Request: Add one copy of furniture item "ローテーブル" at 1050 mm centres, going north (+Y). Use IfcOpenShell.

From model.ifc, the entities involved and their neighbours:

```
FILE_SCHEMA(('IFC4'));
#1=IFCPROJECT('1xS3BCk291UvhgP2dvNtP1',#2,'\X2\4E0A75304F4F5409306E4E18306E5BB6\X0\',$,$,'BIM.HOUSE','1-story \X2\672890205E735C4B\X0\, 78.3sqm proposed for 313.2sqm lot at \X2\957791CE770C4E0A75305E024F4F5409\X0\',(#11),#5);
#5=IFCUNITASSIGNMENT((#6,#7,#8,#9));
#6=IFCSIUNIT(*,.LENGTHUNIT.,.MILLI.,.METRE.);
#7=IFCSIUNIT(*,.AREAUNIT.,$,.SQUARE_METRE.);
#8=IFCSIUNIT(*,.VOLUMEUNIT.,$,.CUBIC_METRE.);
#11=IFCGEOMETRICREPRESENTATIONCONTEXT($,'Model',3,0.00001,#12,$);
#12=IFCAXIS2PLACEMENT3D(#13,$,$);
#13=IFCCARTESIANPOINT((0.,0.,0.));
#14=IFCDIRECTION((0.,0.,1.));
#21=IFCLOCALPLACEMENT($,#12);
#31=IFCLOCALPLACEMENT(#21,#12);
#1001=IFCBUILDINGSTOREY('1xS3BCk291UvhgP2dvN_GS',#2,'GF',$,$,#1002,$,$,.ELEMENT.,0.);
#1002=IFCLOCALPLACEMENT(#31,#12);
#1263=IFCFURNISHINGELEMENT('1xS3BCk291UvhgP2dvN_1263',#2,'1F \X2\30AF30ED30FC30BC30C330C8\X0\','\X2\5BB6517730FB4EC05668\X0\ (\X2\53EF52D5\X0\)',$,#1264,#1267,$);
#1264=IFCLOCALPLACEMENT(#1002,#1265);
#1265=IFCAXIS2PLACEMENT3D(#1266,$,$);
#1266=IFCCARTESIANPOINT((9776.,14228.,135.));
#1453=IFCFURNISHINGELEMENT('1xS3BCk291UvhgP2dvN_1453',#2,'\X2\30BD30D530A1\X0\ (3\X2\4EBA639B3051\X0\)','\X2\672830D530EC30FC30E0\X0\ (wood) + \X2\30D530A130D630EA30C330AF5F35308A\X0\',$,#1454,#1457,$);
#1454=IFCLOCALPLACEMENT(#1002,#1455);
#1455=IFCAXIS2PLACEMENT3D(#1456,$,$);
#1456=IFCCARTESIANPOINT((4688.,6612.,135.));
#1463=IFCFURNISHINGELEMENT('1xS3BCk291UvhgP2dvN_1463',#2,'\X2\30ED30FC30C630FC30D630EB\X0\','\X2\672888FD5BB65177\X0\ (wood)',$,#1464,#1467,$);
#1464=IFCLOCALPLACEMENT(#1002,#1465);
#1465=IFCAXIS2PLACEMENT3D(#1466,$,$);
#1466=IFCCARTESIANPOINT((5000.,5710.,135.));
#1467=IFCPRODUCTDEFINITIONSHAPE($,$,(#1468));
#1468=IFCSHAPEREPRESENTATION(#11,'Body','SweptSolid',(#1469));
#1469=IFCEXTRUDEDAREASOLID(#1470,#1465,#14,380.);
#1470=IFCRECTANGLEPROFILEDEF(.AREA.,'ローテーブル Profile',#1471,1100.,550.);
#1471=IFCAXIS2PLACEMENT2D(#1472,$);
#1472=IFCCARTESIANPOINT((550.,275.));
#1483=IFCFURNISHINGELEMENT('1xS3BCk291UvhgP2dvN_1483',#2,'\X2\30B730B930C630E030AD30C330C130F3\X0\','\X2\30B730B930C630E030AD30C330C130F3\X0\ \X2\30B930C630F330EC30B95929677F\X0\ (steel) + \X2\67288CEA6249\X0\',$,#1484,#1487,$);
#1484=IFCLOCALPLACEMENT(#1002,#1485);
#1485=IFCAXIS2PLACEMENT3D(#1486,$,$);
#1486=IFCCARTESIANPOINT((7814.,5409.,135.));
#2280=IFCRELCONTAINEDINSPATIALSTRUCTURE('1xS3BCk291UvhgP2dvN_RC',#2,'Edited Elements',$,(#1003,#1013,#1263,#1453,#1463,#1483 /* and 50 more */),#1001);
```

```python
import numpy as np
import ifcopenshell
import ifcopenshell.api.geometry
import ifcopenshell.api.root
import ifcopenshell.util.element
import ifcopenshell.util.placement
import ifcopenshell.util.unit

model = ifcopenshell.open("model.ifc")
unit_scale = ifcopenshell.util.unit.calculate_unit_scale(model)


def reuse_history(source, copy):
    """copy_class also copies each property set's owner history, people and application; keep the originals."""
    for rel in copy.IsDefinedBy:
        if rel.is_a("IfcRelDefinesByProperties") and (history := rel.RelatingPropertyDefinition.OwnerHistory):
            rel.RelatingPropertyDefinition.OwnerHistory = source.OwnerHistory
            ifcopenshell.util.element.remove_deep2(model, history)


source = model.by_id(1463)
base = ifcopenshell.util.placement.get_local_placement(source.ObjectPlacement)
step = np.array([0.0, 1.0, 0.0]) * 1.05 / unit_scale

for i in range(1, 2):
    copy = ifcopenshell.api.root.copy_class(model, product=source)
    copy.Representation = ifcopenshell.util.element.copy_deep(
        model, source.Representation, exclude=["IfcGeometricRepresentationContext", "IfcRepresentationMap"]
    )
    reuse_history(source, copy)
    matrix = base.copy()
    matrix[:3, 3] += i * step
    print("added at", matrix[:3, 3].round(3) + 0.0)
    ifcopenshell.api.geometry.edit_object_placement(model, product=copy, matrix=matrix, is_si=False)

model.write("model_updated.ifc")
```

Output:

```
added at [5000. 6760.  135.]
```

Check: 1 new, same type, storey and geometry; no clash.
